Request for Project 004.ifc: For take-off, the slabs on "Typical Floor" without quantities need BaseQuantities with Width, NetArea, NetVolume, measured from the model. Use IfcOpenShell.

First a look at what the model holds.

```python
import ifcopenshell
import ifcopenshell.util.element
import ifcopenshell.util.unit

model = ifcopenshell.open("Project 004.ifc")
print(model.schema)
for unit_type in ("LENGTHUNIT", "AREAUNIT", "VOLUMEUNIT"):
    print(unit_type, ifcopenshell.util.unit.calculate_unit_scale(model, unit_type))
storey = next(s for s in model.by_type("IfcBuildingStorey") if s.Name == "Typical Floor")
slabs = [e for e in ifcopenshell.util.element.get_decomposition(storey) if e.is_a("IfcSlab")]
for e in sorted(slabs, key=lambda e: e.id()):
    print(e.id(), e.is_a(), e.Name, list(ifcopenshell.util.element.get_psets(e, qtos_only=True)), sep=" | ")
```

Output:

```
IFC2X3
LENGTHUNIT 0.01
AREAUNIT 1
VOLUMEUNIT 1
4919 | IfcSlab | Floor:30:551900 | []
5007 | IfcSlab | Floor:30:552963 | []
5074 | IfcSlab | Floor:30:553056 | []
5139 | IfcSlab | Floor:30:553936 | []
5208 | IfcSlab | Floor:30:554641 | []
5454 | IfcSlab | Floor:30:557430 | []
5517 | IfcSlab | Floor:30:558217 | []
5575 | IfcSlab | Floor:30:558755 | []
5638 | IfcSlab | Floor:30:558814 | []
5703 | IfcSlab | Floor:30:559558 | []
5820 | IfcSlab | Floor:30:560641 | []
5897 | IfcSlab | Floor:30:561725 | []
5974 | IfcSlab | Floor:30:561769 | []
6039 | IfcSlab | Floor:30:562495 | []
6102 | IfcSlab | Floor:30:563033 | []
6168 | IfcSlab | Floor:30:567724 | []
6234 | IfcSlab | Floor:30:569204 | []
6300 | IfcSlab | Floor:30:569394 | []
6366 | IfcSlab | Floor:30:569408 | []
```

```python
import ifcopenshell
import ifcopenshell.api.pset
import ifcopenshell.geom
import ifcopenshell.util.element
import ifcopenshell.util.shape
import ifcopenshell.util.unit

model = ifcopenshell.open("Project 004.ifc")
unit_scale = ifcopenshell.util.unit.calculate_unit_scale(model)
area_scale = ifcopenshell.util.unit.calculate_unit_scale(model, "AREAUNIT")
volume_scale = ifcopenshell.util.unit.calculate_unit_scale(model, "VOLUMEUNIT")
settings = ifcopenshell.geom.settings()

storey = next(s for s in model.by_type("IfcBuildingStorey") if s.Name == "Typical Floor")
slabs = [e for e in ifcopenshell.util.element.get_decomposition(storey) if e.is_a("IfcSlab")]

for e in sorted(slabs, key=lambda e: e.id()):
    if ifcopenshell.util.element.get_psets(e, qtos_only=True, should_inherit=False):
        continue
    # Geometry comes back in metres, in the element's own axes.
    shape = ifcopenshell.geom.create_shape(settings, e)
    values = {
        "Width": ifcopenshell.util.shape.get_z(shape.geometry) / unit_scale,
        "NetArea": ifcopenshell.util.shape.get_footprint_area(shape.geometry) / area_scale,
        "NetVolume": ifcopenshell.util.shape.get_volume(shape.geometry) / volume_scale,
    }
    qto = ifcopenshell.api.pset.add_qto(model, product=e, name="BaseQuantities")
    ifcopenshell.api.pset.edit_qto(model, qto=qto, properties=values)
    print(e.id(), {k: round(v, 3) for k, v in values.items()})

model.write("Project 004_v2.ifc")
```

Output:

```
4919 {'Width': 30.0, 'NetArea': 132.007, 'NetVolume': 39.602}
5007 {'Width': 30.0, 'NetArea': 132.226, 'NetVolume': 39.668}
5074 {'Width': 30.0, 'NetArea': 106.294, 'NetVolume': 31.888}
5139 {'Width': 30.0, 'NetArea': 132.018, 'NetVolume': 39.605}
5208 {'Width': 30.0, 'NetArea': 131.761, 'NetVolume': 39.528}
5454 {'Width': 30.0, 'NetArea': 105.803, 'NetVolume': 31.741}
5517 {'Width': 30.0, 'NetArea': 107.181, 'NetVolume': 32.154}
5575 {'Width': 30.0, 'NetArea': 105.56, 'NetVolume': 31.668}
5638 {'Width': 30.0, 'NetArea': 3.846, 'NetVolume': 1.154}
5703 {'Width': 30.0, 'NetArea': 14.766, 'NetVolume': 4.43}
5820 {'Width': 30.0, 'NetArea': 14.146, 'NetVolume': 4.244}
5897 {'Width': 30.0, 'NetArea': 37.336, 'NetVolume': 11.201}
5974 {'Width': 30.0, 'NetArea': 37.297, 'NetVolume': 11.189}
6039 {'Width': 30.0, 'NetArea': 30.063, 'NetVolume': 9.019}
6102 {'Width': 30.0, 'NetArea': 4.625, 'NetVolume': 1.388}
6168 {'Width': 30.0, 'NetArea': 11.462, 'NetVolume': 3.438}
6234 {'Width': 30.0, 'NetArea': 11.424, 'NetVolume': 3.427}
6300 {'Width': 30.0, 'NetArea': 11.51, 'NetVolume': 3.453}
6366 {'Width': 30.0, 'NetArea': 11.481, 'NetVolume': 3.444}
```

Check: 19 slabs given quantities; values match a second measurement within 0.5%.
